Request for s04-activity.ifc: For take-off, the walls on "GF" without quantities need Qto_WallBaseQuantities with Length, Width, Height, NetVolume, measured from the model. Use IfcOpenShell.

First a look at what the model holds.

```python
import ifcopenshell
import ifcopenshell.util.element
import ifcopenshell.util.unit

model = ifcopenshell.open("s04-activity.ifc")
print(model.schema)
for unit_type in ("LENGTHUNIT", "AREAUNIT", "VOLUMEUNIT"):
    print(unit_type, ifcopenshell.util.unit.calculate_unit_scale(model, unit_type))
storey = next(s for s in model.by_type("IfcBuildingStorey") if s.Name == "GF")
walls = [e for e in ifcopenshell.util.element.get_decomposition(storey) if e.is_a("IfcWall")]
for e in sorted(walls, key=lambda e: e.id()):
    print(e.id(), e.is_a(), e.Name, list(ifcopenshell.util.element.get_psets(e, qtos_only=True)), sep=" | ")
```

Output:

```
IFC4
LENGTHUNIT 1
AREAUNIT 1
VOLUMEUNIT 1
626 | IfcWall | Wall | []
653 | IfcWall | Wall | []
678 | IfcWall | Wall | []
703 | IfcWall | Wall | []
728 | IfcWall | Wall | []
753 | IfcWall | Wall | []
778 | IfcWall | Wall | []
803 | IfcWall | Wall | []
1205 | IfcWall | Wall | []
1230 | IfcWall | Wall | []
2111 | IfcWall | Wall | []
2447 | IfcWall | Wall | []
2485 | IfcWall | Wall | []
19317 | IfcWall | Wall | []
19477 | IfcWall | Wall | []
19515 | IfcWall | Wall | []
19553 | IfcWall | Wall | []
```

```python
import ifcopenshell
import ifcopenshell.api.pset
import ifcopenshell.geom
import ifcopenshell.util.element
import ifcopenshell.util.shape
import ifcopenshell.util.unit

model = ifcopenshell.open("s04-activity.ifc")
unit_scale = ifcopenshell.util.unit.calculate_unit_scale(model)
volume_scale = ifcopenshell.util.unit.calculate_unit_scale(model, "VOLUMEUNIT")
settings = ifcopenshell.geom.settings()

storey = next(s for s in model.by_type("IfcBuildingStorey") if s.Name == "GF")
walls = [e for e in ifcopenshell.util.element.get_decomposition(storey) if e.is_a("IfcWall")]

for e in sorted(walls, key=lambda e: e.id()):
    if ifcopenshell.util.element.get_psets(e, qtos_only=True, should_inherit=False):
        continue
    # Geometry comes back in metres, in the element's own axes.
    shape = ifcopenshell.geom.create_shape(settings, e)
    values = {
        "Length": ifcopenshell.util.shape.get_x(shape.geometry) / unit_scale,
        "Width": ifcopenshell.util.shape.get_y(shape.geometry) / unit_scale,
        "Height": ifcopenshell.util.shape.get_z(shape.geometry) / unit_scale,
        "NetVolume": ifcopenshell.util.shape.get_volume(shape.geometry) / volume_scale,
    }
    qto = ifcopenshell.api.pset.add_qto(model, product=e, name="Qto_WallBaseQuantities")
    ifcopenshell.api.pset.edit_qto(model, qto=qto, properties=values)
    print(e.id(), {k: round(v, 3) for k, v in values.items()})

model.write("s04-activity_edited.ifc")
```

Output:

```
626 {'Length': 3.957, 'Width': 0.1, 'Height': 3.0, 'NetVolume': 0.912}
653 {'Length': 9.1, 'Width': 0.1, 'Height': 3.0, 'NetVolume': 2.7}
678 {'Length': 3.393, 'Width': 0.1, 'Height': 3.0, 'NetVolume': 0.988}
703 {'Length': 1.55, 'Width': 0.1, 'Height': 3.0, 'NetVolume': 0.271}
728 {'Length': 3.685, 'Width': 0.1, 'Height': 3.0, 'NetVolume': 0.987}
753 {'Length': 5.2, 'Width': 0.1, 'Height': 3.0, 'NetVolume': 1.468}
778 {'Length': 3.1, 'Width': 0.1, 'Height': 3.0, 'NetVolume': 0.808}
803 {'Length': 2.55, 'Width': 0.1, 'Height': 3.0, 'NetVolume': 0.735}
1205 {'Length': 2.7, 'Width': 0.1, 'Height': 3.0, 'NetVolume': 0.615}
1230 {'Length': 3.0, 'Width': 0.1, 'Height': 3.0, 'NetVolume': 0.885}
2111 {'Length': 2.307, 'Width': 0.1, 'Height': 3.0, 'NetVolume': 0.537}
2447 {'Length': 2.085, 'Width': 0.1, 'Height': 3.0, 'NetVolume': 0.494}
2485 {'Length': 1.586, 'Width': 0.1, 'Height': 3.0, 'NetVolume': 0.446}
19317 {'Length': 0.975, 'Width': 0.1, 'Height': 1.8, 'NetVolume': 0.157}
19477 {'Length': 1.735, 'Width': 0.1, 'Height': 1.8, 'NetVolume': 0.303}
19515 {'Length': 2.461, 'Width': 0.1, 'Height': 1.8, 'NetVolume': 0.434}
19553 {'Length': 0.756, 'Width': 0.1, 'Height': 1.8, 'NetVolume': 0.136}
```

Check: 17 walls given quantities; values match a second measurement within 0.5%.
